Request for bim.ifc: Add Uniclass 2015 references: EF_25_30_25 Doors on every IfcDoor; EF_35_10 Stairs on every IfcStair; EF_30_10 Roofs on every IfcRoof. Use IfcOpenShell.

First a look at what the model holds.

```python
import ifcopenshell

model = ifcopenshell.open("bim.ifc")
print(model.schema)
print("classifications:", [c.Name for c in model.by_type("IfcClassification")])
for ifc_class in ("IfcDoor", "IfcRoof", "IfcStair", "IfcWall", "IfcWindow"):
    print(ifc_class, len(model.by_type(ifc_class)))
```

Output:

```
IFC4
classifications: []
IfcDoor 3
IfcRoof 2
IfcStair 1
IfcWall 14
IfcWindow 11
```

```python
import ifcopenshell
import ifcopenshell.api.classification

model = ifcopenshell.open("bim.ifc")

system = ifcopenshell.api.classification.add_classification(model, classification="Uniclass 2015")

codes = {
    "IfcDoor": ("EF_25_30_25", "Doors"),
    "IfcStair": ("EF_35_10", "Stairs"),
    "IfcRoof": ("EF_30_10", "Roofs"),
}
for ifc_class, (code, name) in codes.items():
    products = model.by_type(ifc_class)
    ifcopenshell.api.classification.add_reference(
        model, products=products, classification=system, identification=code, name=name
    )
    print(code, len(products))

model.write("bim_updated.ifc")
```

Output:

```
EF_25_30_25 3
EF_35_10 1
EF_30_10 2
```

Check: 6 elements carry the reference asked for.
